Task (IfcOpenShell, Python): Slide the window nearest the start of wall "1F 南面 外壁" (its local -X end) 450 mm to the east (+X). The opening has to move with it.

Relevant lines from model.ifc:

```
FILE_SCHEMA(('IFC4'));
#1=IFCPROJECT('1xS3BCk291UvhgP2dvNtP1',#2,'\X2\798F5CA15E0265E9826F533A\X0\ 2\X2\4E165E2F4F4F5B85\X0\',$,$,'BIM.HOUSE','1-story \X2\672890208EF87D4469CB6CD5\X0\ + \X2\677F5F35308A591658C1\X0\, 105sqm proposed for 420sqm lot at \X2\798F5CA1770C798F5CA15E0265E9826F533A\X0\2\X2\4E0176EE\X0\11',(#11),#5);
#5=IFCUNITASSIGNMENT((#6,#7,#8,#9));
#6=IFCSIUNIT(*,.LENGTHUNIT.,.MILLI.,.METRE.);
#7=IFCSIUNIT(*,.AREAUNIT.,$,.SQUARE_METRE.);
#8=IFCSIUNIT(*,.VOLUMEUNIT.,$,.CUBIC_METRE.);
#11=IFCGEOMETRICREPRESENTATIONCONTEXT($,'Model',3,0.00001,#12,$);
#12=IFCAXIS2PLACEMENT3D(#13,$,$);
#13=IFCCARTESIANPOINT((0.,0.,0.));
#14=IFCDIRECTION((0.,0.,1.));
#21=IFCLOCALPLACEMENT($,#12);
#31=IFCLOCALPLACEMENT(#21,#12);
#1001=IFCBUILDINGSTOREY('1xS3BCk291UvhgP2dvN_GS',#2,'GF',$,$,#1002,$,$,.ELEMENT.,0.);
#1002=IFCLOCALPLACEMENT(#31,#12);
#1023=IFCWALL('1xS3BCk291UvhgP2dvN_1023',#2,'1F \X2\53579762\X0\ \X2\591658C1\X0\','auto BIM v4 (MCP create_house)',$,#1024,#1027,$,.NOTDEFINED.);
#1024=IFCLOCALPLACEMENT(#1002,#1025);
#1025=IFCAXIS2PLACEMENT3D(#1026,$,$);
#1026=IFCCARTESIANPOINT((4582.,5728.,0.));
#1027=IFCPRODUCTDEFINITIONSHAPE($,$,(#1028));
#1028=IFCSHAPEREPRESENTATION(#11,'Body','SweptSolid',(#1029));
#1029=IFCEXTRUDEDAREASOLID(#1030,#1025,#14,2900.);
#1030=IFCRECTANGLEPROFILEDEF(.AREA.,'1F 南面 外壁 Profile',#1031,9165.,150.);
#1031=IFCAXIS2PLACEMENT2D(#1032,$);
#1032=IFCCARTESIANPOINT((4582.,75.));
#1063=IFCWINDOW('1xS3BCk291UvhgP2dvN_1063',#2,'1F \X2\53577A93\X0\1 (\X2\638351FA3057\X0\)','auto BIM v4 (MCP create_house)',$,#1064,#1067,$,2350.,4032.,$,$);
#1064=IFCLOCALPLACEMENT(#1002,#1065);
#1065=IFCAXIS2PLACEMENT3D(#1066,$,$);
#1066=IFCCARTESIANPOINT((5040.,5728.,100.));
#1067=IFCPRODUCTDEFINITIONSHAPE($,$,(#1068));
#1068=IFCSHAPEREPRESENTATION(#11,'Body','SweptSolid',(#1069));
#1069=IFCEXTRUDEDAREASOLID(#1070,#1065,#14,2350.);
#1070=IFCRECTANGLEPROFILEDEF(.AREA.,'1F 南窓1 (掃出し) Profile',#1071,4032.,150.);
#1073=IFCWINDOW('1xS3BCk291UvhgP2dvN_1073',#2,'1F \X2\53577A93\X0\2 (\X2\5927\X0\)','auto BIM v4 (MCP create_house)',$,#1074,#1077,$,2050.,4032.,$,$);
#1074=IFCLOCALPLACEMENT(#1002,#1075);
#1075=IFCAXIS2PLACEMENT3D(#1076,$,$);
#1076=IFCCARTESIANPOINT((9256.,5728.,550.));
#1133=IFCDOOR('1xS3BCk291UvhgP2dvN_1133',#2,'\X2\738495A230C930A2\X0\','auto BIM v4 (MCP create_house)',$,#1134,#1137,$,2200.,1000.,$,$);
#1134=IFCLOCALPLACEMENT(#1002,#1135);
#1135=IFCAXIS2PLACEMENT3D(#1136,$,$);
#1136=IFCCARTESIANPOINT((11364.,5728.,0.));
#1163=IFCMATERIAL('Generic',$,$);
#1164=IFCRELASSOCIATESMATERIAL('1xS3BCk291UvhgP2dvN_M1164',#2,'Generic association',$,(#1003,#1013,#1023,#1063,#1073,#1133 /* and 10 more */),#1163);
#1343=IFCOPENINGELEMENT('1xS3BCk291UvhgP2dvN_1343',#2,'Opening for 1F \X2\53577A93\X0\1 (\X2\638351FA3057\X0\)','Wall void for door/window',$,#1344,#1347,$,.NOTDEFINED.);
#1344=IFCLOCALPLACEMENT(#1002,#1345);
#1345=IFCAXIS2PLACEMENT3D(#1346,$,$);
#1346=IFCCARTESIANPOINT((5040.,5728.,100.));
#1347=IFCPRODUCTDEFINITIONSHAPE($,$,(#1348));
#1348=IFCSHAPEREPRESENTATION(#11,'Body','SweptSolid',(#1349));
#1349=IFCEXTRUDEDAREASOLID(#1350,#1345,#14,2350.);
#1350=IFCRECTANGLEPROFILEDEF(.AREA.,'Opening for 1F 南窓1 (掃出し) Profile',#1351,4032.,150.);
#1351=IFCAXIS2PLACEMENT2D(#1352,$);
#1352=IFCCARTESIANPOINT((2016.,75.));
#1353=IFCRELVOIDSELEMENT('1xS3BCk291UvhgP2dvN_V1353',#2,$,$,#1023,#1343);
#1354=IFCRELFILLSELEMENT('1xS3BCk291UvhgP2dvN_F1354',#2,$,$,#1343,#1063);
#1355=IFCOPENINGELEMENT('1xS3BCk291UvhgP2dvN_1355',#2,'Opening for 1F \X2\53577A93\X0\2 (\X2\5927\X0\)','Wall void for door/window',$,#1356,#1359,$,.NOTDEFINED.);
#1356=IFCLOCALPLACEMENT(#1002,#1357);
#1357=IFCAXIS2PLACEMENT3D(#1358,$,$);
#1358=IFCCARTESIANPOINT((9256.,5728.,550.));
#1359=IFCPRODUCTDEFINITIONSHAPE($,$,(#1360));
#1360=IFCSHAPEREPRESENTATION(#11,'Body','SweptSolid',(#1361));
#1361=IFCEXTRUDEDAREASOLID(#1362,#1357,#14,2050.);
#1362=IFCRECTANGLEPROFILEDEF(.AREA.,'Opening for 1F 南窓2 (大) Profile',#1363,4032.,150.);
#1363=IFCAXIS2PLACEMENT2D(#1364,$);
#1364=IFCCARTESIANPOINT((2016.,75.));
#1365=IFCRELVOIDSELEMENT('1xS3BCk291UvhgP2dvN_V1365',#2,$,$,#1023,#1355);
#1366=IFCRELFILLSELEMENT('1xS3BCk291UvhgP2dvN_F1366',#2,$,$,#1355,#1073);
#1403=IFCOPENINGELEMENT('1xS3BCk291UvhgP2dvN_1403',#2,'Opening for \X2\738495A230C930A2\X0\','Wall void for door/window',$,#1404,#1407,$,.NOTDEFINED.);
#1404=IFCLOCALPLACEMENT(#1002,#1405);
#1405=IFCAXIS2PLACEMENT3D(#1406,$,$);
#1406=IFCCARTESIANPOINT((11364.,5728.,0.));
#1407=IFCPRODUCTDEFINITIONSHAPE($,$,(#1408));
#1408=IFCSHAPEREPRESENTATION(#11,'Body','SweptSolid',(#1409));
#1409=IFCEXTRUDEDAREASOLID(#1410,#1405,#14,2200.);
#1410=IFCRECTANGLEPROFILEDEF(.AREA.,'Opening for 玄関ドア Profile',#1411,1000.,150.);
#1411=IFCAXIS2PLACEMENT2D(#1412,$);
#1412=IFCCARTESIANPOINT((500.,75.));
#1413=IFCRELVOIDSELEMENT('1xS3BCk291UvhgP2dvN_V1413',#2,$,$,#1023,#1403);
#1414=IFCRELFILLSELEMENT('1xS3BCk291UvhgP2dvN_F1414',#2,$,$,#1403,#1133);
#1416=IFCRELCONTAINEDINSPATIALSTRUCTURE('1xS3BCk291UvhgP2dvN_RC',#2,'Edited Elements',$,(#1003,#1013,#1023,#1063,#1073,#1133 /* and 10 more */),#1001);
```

```python
import ifcopenshell
import ifcopenshell.api.geometry
import ifcopenshell.util.placement
import ifcopenshell.util.unit

model = ifcopenshell.open("model.ifc")
unit_scale = ifcopenshell.util.unit.calculate_unit_scale(model)

window = model.by_id(1063)
opening = window.FillsVoids[0].RelatingOpeningElement
wall = opening.VoidsElements[0].RelatingBuildingElement

wall_matrix = ifcopenshell.util.placement.get_local_placement(wall.ObjectPlacement)
shift = wall_matrix[:3, 0] * 0.45 / unit_scale
before = ifcopenshell.util.placement.get_local_placement(window.ObjectPlacement)[:3, 3].copy()

# The window is not placed relative to its opening, so move both.
for product in (opening, window):
    matrix = ifcopenshell.util.placement.get_local_placement(product.ObjectPlacement)
    matrix[:3, 3] += shift
    ifcopenshell.api.geometry.edit_object_placement(model, product=product, matrix=matrix, is_si=False)

after = ifcopenshell.util.placement.get_local_placement(window.ObjectPlacement)[:3, 3]
print("window moved by", (after - before).round(3) + 0.0)

model.write("model_rev.ifc")
```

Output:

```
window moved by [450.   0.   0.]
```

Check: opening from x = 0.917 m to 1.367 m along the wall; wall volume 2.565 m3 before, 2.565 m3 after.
